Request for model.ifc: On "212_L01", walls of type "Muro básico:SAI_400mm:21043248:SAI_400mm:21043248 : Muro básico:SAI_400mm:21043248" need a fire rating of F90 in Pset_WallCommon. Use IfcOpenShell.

First a look at what the model holds.

```python
import ifcopenshell
import ifcopenshell.util.element

model = ifcopenshell.open("model.ifc")
print(model.schema)
storey = next(s for s in model.by_type("IfcBuildingStorey") if s.Name == "212_L01")
walls = [e for e in ifcopenshell.util.element.get_decomposition(storey) if e.is_a("IfcWall")]
seen = {}
for e in walls:
    element_type = ifcopenshell.util.element.get_type(e)
    key = (element_type.Name if element_type != e and element_type else None, ifcopenshell.util.element.get_pset(e, "Pset_WallCommon", "FireRating"))
    seen[key] = seen.get(key, 0) + 1
for (name, value), count in sorted(seen.items(), key=str):
    print(count, "x", name, "|", value)
```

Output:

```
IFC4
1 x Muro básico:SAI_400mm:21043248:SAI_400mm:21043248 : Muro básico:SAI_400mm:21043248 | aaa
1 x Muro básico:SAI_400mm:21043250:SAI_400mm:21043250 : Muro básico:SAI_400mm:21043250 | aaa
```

```python
import ifcopenshell
import ifcopenshell.api.pset
import ifcopenshell.util.element

model = ifcopenshell.open("model.ifc")

storey = next(s for s in model.by_type("IfcBuildingStorey") if s.Name == "212_L01")
walls = [e for e in ifcopenshell.util.element.get_decomposition(storey) if e.is_a("IfcWall")]

count = 0
for e in walls:
    element_type = ifcopenshell.util.element.get_type(e)
    if element_type in (None, e) or element_type.Name != "Muro básico:SAI_400mm:21043248:SAI_400mm:21043248 : Muro básico:SAI_400mm:21043248":
        continue
    # add_pset returns the element's existing set when there is one.
    pset = ifcopenshell.api.pset.add_pset(model, product=e, name="Pset_WallCommon")
    ifcopenshell.api.pset.edit_pset(model, pset=pset, properties={"FireRating": "F90"})
    count += 1

print(count, "walls updated")

model.write("model_rev.ifc")
```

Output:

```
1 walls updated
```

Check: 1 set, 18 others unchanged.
